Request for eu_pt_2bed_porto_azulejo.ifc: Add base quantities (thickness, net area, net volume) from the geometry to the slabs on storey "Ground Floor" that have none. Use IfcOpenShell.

First a look at what the model holds.

```python
import ifcopenshell
import ifcopenshell.util.element
import ifcopenshell.util.unit

model = ifcopenshell.open("eu_pt_2bed_porto_azulejo.ifc")
print(model.schema)
for unit_type in ("LENGTHUNIT", "AREAUNIT", "VOLUMEUNIT"):
    print(unit_type, ifcopenshell.util.unit.calculate_unit_scale(model, unit_type))
storey = next(s for s in model.by_type("IfcBuildingStorey") if s.Name == "Ground Floor")
slabs = [e for e in ifcopenshell.util.element.get_decomposition(storey) if e.is_a("IfcSlab")]
for e in sorted(slabs, key=lambda e: e.id()):
    print(e.id(), e.is_a(), e.Name, list(ifcopenshell.util.element.get_psets(e, qtos_only=True)), sep=" | ")
```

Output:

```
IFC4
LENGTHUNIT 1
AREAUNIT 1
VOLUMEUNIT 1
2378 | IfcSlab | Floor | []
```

```python
import ifcopenshell
import ifcopenshell.api.pset
import ifcopenshell.geom
import ifcopenshell.util.element
import ifcopenshell.util.shape
import ifcopenshell.util.unit

model = ifcopenshell.open("eu_pt_2bed_porto_azulejo.ifc")
unit_scale = ifcopenshell.util.unit.calculate_unit_scale(model)
area_scale = ifcopenshell.util.unit.calculate_unit_scale(model, "AREAUNIT")
volume_scale = ifcopenshell.util.unit.calculate_unit_scale(model, "VOLUMEUNIT")
settings = ifcopenshell.geom.settings()

storey = next(s for s in model.by_type("IfcBuildingStorey") if s.Name == "Ground Floor")
slabs = [e for e in ifcopenshell.util.element.get_decomposition(storey) if e.is_a("IfcSlab")]

for e in sorted(slabs, key=lambda e: e.id()):
    if ifcopenshell.util.element.get_psets(e, qtos_only=True, should_inherit=False):
        continue
    # Geometry comes back in metres, in the element's own axes.
    shape = ifcopenshell.geom.create_shape(settings, e)
    values = {
        "Width": ifcopenshell.util.shape.get_z(shape.geometry) / unit_scale,
        "NetArea": ifcopenshell.util.shape.get_footprint_area(shape.geometry) / area_scale,
        "NetVolume": ifcopenshell.util.shape.get_volume(shape.geometry) / volume_scale,
    }
    qto = ifcopenshell.api.pset.add_qto(model, product=e, name="Qto_SlabBaseQuantities")
    ifcopenshell.api.pset.edit_qto(model, qto=qto, properties=values)
    print(e.id(), {k: round(v, 3) for k, v in values.items()})

model.write("eu_pt_2bed_porto_azulejo_updated.ifc")
```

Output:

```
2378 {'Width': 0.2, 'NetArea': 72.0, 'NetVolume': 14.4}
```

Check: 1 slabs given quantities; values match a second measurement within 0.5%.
